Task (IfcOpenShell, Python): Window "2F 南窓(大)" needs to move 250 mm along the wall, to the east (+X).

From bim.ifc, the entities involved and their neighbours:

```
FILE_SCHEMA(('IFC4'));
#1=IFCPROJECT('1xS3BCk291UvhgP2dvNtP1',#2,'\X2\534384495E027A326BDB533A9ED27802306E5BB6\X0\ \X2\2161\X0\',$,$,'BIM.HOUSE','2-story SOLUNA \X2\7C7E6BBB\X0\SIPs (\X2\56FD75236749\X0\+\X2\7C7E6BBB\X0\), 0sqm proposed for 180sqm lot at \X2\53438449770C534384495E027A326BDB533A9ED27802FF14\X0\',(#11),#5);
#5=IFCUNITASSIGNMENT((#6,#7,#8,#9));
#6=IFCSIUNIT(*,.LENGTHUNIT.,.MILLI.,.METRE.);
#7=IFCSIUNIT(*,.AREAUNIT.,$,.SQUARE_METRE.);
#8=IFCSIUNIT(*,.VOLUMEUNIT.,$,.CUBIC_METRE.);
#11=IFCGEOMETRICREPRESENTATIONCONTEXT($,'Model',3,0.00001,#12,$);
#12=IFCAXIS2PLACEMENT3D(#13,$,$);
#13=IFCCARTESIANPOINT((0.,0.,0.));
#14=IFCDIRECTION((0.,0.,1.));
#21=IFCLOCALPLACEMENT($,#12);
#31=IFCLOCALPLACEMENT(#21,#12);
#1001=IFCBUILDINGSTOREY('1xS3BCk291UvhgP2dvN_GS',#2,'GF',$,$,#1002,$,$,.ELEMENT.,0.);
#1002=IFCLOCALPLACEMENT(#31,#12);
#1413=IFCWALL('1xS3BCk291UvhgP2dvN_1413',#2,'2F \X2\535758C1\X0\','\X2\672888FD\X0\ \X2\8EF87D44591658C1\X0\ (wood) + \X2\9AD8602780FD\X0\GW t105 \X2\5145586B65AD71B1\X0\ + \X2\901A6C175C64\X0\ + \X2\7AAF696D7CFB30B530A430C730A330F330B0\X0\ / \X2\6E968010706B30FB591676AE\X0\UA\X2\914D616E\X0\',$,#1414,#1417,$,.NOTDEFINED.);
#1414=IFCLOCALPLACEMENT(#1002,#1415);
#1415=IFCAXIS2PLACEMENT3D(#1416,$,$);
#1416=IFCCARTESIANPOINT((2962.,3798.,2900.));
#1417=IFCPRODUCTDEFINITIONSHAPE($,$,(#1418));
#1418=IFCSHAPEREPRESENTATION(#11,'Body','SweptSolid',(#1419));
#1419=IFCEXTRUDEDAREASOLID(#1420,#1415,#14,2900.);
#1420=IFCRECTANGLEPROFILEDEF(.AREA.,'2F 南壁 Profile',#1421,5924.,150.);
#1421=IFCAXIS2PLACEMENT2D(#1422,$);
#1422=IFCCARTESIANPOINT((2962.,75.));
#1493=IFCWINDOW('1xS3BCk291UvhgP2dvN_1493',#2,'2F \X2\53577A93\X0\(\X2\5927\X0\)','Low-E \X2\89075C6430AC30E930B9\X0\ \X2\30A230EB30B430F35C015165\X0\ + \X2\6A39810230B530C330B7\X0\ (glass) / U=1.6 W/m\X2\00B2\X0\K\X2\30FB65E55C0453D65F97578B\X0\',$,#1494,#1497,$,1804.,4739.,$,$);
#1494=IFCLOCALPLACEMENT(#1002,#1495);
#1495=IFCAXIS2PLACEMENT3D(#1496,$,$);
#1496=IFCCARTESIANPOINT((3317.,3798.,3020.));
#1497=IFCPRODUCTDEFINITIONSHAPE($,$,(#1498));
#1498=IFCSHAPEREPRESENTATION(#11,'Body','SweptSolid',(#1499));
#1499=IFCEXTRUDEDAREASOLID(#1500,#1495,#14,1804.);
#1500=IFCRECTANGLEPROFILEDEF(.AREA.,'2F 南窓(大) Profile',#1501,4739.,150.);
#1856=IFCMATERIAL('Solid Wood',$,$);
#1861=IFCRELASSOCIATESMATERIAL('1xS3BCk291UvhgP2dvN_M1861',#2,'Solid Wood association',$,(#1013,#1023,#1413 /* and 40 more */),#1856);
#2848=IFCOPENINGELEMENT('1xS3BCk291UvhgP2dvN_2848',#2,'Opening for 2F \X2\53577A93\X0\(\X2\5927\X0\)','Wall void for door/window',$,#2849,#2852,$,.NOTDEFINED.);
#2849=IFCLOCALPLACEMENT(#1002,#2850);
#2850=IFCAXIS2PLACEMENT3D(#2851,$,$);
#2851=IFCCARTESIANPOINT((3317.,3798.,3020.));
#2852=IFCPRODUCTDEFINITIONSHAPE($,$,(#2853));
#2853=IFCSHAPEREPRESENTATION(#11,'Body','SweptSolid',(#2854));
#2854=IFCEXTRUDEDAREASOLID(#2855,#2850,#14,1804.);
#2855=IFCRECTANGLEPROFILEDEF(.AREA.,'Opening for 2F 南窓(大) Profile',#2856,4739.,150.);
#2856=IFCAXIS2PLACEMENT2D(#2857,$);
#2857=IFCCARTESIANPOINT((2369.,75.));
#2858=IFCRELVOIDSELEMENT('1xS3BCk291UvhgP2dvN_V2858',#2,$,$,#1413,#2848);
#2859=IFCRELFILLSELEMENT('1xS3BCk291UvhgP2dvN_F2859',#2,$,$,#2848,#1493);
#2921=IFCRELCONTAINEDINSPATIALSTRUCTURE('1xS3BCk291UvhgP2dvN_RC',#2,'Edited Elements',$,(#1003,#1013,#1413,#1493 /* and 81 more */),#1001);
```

```python
import ifcopenshell
import ifcopenshell.api.geometry
import ifcopenshell.util.placement
import ifcopenshell.util.unit

model = ifcopenshell.open("bim.ifc")
unit_scale = ifcopenshell.util.unit.calculate_unit_scale(model)

window = model.by_guid("1xS3BCk291UvhgP2dvN_1493")
opening = window.FillsVoids[0].RelatingOpeningElement
wall = opening.VoidsElements[0].RelatingBuildingElement

wall_matrix = ifcopenshell.util.placement.get_local_placement(wall.ObjectPlacement)
shift = wall_matrix[:3, 0] * 0.25 / unit_scale
before = ifcopenshell.util.placement.get_local_placement(window.ObjectPlacement)[:3, 3].copy()

# The window is not placed relative to its opening, so move both.
for product in (opening, window):
    matrix = ifcopenshell.util.placement.get_local_placement(product.ObjectPlacement)
    matrix[:3, 3] += shift
    ifcopenshell.api.geometry.edit_object_placement(model, product=product, matrix=matrix, is_si=False)

after = ifcopenshell.util.placement.get_local_placement(window.ObjectPlacement)[:3, 3]
print("window moved by", (after - before).round(3) + 0.0)

model.write("bim-out.ifc")
```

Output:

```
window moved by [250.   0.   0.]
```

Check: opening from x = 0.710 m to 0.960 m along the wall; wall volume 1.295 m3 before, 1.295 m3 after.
